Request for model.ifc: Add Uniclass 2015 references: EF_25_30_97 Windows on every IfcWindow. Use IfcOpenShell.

First a look at what the model holds.

```python
import ifcopenshell

model = ifcopenshell.open("model.ifc")
print(model.schema)
print("classifications:", [c.Name for c in model.by_type("IfcClassification")])
for ifc_class in ("IfcDoor", "IfcRoof", "IfcStair", "IfcWall", "IfcWindow"):
    print(ifc_class, len(model.by_type(ifc_class)))
```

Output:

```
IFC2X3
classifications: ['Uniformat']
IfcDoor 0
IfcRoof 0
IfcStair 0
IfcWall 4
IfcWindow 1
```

```python
import ifcopenshell
import ifcopenshell.api.classification

model = ifcopenshell.open("model.ifc")

# IFC2X3 requires Source and Edition and has no link from the project to the system.
system = model.create_entity("IfcClassification", Source="NBS", Edition="2015", Name="Uniclass 2015")

codes = {
    "IfcWindow": ("EF_25_30_97", "Windows"),
}
for ifc_class, (code, name) in codes.items():
    products = model.by_type(ifc_class)
    ifcopenshell.api.classification.add_reference(
        model, products=products, classification=system, identification=code, name=name
    )
    print(code, len(products))

model.write("model-out.ifc")
```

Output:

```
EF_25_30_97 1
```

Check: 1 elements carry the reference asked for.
